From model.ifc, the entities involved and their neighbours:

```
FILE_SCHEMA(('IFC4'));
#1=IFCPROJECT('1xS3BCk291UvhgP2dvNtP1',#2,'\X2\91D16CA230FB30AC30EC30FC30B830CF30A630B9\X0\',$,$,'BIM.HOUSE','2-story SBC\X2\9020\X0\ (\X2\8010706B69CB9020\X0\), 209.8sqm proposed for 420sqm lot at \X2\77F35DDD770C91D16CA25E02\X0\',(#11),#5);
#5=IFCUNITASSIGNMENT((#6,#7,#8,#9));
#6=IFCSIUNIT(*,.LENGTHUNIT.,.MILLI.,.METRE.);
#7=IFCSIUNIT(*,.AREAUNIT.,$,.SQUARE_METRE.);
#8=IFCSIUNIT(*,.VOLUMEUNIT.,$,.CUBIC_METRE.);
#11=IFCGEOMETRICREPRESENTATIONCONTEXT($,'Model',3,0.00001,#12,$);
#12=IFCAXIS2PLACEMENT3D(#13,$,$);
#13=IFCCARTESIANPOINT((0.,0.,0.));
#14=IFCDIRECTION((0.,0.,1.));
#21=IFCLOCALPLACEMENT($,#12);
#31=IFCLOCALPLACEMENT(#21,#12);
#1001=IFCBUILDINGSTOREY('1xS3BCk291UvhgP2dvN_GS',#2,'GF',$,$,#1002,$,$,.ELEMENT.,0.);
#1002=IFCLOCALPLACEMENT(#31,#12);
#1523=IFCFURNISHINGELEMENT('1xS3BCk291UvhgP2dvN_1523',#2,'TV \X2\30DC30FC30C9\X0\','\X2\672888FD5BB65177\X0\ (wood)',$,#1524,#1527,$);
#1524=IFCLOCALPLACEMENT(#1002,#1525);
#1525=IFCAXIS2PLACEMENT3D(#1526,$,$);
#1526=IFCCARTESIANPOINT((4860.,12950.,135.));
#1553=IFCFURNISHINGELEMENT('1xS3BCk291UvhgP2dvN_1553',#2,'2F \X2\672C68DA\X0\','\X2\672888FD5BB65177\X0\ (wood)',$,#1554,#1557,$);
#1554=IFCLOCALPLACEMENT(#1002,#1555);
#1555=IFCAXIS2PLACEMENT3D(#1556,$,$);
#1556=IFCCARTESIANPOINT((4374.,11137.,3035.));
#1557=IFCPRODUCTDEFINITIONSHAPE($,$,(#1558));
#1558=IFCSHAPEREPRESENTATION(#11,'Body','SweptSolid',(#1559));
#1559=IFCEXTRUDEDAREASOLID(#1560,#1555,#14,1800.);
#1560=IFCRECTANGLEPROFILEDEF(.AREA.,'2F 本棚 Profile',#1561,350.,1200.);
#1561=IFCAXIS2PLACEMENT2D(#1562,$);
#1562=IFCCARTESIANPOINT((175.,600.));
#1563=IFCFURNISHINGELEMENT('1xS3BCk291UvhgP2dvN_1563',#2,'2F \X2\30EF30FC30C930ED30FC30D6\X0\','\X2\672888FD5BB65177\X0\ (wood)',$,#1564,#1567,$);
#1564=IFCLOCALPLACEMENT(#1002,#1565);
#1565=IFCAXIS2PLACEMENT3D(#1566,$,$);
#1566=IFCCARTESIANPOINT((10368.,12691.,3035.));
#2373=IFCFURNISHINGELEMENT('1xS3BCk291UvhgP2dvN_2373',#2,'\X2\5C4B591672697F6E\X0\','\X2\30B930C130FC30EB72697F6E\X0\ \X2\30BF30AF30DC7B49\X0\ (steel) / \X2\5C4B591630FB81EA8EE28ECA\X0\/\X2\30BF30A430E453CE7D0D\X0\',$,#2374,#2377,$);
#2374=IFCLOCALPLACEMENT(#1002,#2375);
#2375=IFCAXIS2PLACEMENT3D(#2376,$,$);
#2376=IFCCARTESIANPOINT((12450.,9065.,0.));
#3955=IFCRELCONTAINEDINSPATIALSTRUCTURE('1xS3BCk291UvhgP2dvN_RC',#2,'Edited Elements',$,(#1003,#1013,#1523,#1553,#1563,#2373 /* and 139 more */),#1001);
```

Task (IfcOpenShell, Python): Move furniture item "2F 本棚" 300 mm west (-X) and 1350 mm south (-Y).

```python
import ifcopenshell
import ifcopenshell.api.geometry
import ifcopenshell.util.placement

model = ifcopenshell.open("model.ifc")

item = model.by_guid("1xS3BCk291UvhgP2dvN_1553")
matrix = ifcopenshell.util.placement.get_local_placement(item.ObjectPlacement)
matrix[0, 3] -= 300.0
matrix[1, 3] -= 1350.0
ifcopenshell.api.geometry.edit_object_placement(model, product=item, matrix=matrix, is_si=False)

print(ifcopenshell.util.placement.get_local_placement(item.ObjectPlacement).round(3) + 0.0)

model.write("model_rev.ifc")
```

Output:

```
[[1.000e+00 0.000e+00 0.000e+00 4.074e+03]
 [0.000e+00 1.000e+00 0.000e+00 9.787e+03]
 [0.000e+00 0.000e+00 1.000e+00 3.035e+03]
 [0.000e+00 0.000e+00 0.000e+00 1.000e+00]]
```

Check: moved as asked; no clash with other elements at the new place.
